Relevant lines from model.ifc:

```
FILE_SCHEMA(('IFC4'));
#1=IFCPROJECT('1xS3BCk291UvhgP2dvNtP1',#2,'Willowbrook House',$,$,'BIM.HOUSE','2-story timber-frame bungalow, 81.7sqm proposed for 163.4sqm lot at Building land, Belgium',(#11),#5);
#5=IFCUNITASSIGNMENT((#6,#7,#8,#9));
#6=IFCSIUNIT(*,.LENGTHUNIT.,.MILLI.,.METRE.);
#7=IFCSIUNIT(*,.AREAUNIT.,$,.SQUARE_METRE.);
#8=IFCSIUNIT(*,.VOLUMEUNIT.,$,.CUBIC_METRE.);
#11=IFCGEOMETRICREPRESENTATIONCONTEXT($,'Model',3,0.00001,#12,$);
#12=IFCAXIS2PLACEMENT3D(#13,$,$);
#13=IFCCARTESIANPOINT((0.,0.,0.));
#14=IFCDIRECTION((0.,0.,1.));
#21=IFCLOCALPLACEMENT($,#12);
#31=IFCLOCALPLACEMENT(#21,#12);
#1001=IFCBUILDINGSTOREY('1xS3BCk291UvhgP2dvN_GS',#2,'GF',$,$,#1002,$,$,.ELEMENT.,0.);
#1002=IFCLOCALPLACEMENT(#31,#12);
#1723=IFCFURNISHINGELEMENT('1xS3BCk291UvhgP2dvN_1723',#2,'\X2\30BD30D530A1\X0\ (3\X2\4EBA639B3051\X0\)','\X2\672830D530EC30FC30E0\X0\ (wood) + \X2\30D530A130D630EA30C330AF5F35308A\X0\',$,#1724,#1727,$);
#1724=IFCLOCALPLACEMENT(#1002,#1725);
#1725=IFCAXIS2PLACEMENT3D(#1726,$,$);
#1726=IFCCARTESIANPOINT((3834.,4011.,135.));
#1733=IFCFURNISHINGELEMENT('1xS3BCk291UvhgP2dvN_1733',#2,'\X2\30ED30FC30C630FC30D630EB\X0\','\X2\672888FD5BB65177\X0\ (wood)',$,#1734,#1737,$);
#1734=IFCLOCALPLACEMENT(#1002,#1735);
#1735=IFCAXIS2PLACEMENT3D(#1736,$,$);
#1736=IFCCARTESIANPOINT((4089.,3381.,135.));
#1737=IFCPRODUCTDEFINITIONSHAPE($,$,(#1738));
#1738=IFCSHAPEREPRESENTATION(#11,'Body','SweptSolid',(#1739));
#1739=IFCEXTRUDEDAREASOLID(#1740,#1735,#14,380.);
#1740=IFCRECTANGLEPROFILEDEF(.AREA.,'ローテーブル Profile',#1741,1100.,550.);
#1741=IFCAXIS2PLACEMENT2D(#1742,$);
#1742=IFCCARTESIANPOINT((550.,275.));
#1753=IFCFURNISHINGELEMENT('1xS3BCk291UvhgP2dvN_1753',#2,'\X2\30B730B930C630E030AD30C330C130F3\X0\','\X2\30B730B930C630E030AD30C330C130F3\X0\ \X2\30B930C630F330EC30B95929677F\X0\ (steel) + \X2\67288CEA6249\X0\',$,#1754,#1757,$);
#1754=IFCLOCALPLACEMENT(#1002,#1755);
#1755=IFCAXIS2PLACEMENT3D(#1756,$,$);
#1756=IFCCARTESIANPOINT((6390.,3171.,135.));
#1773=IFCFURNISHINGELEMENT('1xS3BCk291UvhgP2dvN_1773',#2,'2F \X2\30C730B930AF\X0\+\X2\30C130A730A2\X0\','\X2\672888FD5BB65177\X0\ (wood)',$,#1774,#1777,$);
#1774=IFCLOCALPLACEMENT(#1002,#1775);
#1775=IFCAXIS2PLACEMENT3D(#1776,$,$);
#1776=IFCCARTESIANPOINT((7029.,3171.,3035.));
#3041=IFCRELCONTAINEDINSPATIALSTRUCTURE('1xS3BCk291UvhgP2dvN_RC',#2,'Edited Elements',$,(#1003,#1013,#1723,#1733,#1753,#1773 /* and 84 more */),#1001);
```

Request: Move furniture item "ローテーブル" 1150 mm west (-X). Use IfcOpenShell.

```python
import ifcopenshell
import ifcopenshell.api.geometry
import ifcopenshell.util.placement
import ifcopenshell.util.unit

model = ifcopenshell.open("model.ifc")
unit_scale = ifcopenshell.util.unit.calculate_unit_scale(model)

item = model.by_guid("1xS3BCk291UvhgP2dvN_1733")
matrix = ifcopenshell.util.placement.get_local_placement(item.ObjectPlacement)
matrix[0, 3] -= 1.15 / unit_scale
ifcopenshell.api.geometry.edit_object_placement(model, product=item, matrix=matrix, is_si=False)

print(ifcopenshell.util.placement.get_local_placement(item.ObjectPlacement).round(3) + 0.0)

model.write("model_updated.ifc")
```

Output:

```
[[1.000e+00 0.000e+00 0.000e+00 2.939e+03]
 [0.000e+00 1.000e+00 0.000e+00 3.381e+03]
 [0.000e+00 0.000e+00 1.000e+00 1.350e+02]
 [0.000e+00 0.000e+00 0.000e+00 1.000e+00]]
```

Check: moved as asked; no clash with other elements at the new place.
